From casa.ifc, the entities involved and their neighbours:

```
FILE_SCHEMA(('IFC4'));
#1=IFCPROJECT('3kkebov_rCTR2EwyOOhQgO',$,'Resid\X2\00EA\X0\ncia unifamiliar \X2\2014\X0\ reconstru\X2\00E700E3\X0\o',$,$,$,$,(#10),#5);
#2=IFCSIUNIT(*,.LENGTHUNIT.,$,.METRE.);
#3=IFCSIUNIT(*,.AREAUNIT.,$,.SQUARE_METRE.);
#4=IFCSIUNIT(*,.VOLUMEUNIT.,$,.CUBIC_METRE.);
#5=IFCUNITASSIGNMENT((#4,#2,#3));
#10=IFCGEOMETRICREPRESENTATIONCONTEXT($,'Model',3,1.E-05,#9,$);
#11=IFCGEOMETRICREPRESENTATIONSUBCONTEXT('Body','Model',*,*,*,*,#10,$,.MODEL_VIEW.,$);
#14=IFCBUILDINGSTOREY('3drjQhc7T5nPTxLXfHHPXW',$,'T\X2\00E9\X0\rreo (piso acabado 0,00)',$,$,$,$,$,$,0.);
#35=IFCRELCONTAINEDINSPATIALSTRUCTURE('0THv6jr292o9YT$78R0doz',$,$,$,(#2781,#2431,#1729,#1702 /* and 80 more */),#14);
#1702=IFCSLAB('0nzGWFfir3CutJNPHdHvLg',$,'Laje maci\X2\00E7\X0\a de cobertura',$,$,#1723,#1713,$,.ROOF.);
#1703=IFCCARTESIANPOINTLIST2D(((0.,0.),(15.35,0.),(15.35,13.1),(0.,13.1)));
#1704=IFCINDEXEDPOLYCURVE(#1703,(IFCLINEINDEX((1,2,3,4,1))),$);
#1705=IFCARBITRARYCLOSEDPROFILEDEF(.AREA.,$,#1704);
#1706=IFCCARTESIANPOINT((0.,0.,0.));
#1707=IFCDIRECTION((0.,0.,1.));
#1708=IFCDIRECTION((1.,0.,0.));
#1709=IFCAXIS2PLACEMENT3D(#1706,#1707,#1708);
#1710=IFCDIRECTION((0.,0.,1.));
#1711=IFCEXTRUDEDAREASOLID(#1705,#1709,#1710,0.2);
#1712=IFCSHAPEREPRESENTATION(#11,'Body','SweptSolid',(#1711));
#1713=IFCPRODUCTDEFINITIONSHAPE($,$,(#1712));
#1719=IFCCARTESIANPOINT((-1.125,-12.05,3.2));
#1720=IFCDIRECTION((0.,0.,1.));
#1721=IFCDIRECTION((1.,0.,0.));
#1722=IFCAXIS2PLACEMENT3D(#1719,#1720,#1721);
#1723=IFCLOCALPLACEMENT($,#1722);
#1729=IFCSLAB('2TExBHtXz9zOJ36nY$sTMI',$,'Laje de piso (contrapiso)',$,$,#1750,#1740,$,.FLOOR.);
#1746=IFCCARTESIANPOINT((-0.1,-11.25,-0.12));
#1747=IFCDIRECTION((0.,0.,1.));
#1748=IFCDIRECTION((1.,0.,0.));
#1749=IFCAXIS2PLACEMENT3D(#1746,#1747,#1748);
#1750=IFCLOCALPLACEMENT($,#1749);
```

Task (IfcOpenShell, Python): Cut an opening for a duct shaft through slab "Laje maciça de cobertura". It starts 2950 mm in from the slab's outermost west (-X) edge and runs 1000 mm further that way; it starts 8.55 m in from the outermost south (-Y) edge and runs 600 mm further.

```python
import numpy as np
import ifcopenshell
import ifcopenshell.api.feature
import ifcopenshell.api.geometry
import ifcopenshell.api.root
import ifcopenshell.geom
import ifcopenshell.util.placement
import ifcopenshell.util.representation
import ifcopenshell.util.shape
import ifcopenshell.util.unit

model = ifcopenshell.open("casa.ifc")
unit_scale = ifcopenshell.util.unit.calculate_unit_scale(model)
settings = ifcopenshell.geom.settings()


def volume(element):
    """Net volume in cubic metres, openings subtracted."""
    shape = ifcopenshell.geom.create_shape(settings, element)
    return ifcopenshell.util.shape.get_volume(shape.geometry)


slab = model.by_guid("0nzGWFfir3CutJNPHdHvLg")
before = volume(slab)

# Extent in the slab's own axes, in metres. The edges named are its -X and -Y sides.
slab_shape = ifcopenshell.geom.create_shape(settings, slab)
vertices = ifcopenshell.util.shape.get_vertices(slab_shape.geometry)
x_min, y_min, bottom = vertices.min(axis=0)
top = vertices[:, 2].max()

opening = ifcopenshell.api.root.create_entity(model, ifc_class="IfcOpeningElement", name="Duct shaft opening", predefined_type="OPENING")
context = ifcopenshell.util.representation.get_context(model, "Model", "Body", "MODEL_VIEW")
width, depth = 1, 0.6
outline = [(0.0, 0.0), (width, 0.0), (width, depth), (0.0, depth), (0.0, 0.0)]
# Overshoot both faces by 50 mm so the cut is clean.
shape = ifcopenshell.api.geometry.add_slab_representation(
    model, context=context, depth=top - bottom + 0.1, polyline=outline
)
ifcopenshell.api.geometry.assign_representation(model, product=opening, representation=shape)

matrix = ifcopenshell.util.placement.get_local_placement(slab.ObjectPlacement)
matrix[:, 3] = matrix @ np.append(np.array([x_min + 2.95, y_min + 8.55, bottom - 0.05]) / unit_scale, 1.0)
ifcopenshell.api.geometry.edit_object_placement(model, product=opening, matrix=matrix, is_si=False)
ifcopenshell.api.feature.add_feature(model, feature=opening, element=slab)

after = volume(slab)

print(f"slab volume {before:.3f} -> {after:.3f} m3")

model.write("casa_v2.ifc")
```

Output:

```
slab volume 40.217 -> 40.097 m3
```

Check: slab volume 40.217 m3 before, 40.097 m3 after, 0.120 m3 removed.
